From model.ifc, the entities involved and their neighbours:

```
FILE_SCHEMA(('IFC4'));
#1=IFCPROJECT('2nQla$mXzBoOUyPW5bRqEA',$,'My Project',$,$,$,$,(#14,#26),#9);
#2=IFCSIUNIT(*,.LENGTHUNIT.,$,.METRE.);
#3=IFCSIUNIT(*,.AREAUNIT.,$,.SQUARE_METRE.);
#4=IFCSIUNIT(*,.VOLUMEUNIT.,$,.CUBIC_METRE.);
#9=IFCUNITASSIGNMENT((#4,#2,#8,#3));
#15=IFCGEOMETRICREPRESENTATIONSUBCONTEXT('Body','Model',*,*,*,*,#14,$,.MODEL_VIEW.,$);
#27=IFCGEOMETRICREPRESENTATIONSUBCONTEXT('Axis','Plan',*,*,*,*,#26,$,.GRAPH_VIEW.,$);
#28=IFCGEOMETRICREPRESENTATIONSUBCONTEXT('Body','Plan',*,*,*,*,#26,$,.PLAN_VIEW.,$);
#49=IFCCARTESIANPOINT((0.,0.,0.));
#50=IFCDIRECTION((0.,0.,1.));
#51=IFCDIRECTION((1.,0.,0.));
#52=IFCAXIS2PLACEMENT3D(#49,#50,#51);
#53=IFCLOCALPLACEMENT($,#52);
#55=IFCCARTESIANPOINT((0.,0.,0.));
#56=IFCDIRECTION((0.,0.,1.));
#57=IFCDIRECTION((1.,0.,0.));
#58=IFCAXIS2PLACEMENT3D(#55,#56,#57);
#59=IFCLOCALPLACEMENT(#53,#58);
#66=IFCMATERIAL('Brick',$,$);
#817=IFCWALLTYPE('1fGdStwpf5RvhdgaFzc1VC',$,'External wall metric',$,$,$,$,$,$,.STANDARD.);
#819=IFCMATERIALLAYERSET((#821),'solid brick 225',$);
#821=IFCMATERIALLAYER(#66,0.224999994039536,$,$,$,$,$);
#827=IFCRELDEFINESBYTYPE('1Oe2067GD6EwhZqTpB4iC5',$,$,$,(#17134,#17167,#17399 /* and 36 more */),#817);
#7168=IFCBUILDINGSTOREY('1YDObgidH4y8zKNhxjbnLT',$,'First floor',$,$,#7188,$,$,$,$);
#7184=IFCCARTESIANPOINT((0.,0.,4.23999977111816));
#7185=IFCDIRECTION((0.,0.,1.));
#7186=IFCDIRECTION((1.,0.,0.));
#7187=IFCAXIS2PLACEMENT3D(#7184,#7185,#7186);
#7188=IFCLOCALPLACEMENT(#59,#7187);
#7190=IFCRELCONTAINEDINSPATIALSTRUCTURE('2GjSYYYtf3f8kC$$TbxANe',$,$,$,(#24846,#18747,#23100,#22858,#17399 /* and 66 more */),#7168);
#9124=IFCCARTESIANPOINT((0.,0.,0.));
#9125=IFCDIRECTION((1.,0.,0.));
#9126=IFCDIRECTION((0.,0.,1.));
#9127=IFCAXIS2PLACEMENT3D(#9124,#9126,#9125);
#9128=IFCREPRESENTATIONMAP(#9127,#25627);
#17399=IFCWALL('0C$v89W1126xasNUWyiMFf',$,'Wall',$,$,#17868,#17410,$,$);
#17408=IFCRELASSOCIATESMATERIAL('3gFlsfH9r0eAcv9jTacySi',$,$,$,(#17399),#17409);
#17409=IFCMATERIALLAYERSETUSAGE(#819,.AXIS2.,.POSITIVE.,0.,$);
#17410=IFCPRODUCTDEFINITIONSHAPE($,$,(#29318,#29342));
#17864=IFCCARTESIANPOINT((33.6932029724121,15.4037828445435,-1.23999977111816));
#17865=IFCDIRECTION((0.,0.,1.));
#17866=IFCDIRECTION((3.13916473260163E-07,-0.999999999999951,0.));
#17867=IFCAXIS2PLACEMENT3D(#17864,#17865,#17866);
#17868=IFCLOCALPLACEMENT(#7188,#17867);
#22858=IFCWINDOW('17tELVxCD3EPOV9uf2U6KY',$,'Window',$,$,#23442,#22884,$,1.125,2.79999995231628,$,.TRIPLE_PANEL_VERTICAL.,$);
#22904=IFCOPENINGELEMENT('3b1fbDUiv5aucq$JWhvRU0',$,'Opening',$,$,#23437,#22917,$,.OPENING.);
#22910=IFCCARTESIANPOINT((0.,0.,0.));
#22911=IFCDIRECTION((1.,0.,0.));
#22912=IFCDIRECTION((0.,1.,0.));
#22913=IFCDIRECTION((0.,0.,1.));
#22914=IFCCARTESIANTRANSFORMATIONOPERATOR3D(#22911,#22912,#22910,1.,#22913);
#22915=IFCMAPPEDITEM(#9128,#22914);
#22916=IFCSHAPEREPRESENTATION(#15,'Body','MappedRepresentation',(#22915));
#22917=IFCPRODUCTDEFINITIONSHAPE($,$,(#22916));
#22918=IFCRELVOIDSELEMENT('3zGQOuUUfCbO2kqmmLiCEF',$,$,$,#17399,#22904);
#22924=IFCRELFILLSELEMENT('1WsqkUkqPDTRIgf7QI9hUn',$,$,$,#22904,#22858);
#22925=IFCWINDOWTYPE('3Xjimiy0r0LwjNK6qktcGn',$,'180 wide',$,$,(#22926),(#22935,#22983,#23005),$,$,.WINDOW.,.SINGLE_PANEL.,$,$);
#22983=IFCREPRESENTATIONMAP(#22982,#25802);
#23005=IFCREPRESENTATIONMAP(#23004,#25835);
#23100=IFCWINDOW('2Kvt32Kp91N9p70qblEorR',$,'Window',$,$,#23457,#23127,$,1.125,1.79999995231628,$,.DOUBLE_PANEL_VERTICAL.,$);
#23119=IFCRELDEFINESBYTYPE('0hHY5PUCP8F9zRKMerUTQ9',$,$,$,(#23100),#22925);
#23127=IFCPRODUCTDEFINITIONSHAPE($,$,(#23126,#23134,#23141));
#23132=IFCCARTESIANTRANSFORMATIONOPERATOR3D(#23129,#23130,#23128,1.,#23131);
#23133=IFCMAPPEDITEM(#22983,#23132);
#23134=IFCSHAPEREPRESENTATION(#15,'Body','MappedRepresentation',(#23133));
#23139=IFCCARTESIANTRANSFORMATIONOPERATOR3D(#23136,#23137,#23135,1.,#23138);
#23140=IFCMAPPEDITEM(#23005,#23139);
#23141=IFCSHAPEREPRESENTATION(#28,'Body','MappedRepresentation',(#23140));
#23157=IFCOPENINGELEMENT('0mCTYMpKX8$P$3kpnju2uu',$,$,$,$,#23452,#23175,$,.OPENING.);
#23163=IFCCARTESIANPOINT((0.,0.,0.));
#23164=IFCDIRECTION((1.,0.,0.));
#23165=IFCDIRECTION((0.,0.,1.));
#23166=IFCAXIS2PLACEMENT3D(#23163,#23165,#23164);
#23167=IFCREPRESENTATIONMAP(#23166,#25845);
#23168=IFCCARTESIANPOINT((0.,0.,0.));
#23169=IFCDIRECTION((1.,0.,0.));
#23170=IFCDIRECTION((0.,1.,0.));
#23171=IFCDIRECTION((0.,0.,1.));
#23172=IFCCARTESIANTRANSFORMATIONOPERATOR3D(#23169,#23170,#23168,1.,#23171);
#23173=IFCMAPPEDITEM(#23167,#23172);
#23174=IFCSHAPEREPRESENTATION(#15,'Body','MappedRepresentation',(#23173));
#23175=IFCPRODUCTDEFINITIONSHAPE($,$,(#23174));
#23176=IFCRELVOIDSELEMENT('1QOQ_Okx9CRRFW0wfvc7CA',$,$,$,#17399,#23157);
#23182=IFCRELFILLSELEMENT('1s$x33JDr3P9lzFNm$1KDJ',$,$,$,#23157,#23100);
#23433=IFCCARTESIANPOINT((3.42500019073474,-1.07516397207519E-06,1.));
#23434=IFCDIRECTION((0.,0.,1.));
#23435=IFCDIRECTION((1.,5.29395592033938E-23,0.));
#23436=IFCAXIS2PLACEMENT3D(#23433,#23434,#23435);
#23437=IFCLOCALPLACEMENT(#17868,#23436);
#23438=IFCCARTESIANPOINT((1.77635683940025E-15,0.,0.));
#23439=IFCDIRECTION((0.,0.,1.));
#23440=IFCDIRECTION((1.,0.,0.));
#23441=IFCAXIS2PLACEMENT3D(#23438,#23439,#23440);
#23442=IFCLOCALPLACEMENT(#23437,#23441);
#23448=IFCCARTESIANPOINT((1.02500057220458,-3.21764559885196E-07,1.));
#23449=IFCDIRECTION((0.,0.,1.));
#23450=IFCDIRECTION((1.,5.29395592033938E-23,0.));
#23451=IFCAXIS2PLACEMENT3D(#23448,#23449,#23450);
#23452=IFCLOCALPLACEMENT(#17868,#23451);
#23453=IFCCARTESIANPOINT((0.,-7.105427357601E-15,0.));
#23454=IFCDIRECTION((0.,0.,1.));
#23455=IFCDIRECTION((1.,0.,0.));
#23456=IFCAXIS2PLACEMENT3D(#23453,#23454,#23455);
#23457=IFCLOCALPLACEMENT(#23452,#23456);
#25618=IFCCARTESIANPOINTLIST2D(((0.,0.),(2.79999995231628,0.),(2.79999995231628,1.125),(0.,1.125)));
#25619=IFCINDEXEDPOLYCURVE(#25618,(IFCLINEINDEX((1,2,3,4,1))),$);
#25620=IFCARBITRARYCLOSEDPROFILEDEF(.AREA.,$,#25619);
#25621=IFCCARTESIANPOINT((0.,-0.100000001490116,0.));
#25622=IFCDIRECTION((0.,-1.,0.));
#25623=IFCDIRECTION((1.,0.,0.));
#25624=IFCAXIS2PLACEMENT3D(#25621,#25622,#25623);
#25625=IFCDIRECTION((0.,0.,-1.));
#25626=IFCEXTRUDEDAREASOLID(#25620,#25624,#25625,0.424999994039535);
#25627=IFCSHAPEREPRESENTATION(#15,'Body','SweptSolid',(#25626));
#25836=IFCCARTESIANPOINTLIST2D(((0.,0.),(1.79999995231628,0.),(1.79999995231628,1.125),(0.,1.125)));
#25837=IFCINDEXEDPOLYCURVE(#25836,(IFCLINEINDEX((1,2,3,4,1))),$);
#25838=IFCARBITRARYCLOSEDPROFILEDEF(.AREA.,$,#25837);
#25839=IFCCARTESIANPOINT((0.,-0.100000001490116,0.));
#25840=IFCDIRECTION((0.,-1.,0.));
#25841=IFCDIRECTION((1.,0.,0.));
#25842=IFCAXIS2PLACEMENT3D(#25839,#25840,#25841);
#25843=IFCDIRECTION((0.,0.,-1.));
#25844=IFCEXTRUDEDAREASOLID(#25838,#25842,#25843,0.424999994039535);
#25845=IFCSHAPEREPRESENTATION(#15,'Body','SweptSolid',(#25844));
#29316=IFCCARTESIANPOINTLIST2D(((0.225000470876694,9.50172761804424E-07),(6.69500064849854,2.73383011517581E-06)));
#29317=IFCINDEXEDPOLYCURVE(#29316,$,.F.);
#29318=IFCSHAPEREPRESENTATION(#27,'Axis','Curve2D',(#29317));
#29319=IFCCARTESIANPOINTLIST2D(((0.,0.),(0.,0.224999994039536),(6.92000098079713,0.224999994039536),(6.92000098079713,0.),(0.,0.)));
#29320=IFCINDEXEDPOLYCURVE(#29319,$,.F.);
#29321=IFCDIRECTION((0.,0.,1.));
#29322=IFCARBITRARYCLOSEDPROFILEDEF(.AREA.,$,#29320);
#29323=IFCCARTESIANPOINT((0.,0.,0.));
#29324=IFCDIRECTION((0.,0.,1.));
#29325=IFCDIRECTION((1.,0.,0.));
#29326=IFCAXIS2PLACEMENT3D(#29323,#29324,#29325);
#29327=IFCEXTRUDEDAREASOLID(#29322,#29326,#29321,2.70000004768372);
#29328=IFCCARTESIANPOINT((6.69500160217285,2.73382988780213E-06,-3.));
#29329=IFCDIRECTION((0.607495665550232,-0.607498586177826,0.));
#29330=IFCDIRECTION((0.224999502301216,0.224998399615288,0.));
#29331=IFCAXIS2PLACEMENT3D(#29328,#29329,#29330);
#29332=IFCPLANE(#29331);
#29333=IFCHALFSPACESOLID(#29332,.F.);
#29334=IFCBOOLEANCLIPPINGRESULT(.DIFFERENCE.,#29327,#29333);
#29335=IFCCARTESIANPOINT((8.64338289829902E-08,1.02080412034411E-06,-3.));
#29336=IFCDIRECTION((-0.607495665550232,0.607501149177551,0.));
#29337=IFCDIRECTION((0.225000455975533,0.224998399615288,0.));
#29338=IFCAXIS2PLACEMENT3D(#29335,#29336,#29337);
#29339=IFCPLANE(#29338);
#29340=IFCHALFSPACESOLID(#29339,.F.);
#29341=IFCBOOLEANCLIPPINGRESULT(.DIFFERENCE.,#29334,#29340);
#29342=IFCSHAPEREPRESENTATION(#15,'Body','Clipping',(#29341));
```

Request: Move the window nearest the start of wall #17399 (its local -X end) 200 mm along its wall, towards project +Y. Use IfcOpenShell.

```python
import ifcopenshell
import ifcopenshell.api.geometry
import ifcopenshell.util.placement
import ifcopenshell.util.unit

model = ifcopenshell.open("model.ifc")
unit_scale = ifcopenshell.util.unit.calculate_unit_scale(model)

window = model.by_guid("2Kvt32Kp91N9p70qblEorR")
opening = window.FillsVoids[0].RelatingOpeningElement
wall = opening.VoidsElements[0].RelatingBuildingElement

wall_matrix = ifcopenshell.util.placement.get_local_placement(wall.ObjectPlacement)
shift = wall_matrix[:3, 0] * -0.2 / unit_scale
before = ifcopenshell.util.placement.get_local_placement(window.ObjectPlacement)[:3, 3].copy()

# The window is placed relative to its opening, so it follows when the opening moves.
matrix = ifcopenshell.util.placement.get_local_placement(opening.ObjectPlacement)
matrix[:3, 3] += shift
ifcopenshell.api.geometry.edit_object_placement(
    model, product=opening, matrix=matrix, is_si=False, should_transform_children=True
)

after = ifcopenshell.util.placement.get_local_placement(window.ObjectPlacement)[:3, 3]
print("window moved by", (after - before).round(3) + 0.0)

model.write("model-out.ifc")
```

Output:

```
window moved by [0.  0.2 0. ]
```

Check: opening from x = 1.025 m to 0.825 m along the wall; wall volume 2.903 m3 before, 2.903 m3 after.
